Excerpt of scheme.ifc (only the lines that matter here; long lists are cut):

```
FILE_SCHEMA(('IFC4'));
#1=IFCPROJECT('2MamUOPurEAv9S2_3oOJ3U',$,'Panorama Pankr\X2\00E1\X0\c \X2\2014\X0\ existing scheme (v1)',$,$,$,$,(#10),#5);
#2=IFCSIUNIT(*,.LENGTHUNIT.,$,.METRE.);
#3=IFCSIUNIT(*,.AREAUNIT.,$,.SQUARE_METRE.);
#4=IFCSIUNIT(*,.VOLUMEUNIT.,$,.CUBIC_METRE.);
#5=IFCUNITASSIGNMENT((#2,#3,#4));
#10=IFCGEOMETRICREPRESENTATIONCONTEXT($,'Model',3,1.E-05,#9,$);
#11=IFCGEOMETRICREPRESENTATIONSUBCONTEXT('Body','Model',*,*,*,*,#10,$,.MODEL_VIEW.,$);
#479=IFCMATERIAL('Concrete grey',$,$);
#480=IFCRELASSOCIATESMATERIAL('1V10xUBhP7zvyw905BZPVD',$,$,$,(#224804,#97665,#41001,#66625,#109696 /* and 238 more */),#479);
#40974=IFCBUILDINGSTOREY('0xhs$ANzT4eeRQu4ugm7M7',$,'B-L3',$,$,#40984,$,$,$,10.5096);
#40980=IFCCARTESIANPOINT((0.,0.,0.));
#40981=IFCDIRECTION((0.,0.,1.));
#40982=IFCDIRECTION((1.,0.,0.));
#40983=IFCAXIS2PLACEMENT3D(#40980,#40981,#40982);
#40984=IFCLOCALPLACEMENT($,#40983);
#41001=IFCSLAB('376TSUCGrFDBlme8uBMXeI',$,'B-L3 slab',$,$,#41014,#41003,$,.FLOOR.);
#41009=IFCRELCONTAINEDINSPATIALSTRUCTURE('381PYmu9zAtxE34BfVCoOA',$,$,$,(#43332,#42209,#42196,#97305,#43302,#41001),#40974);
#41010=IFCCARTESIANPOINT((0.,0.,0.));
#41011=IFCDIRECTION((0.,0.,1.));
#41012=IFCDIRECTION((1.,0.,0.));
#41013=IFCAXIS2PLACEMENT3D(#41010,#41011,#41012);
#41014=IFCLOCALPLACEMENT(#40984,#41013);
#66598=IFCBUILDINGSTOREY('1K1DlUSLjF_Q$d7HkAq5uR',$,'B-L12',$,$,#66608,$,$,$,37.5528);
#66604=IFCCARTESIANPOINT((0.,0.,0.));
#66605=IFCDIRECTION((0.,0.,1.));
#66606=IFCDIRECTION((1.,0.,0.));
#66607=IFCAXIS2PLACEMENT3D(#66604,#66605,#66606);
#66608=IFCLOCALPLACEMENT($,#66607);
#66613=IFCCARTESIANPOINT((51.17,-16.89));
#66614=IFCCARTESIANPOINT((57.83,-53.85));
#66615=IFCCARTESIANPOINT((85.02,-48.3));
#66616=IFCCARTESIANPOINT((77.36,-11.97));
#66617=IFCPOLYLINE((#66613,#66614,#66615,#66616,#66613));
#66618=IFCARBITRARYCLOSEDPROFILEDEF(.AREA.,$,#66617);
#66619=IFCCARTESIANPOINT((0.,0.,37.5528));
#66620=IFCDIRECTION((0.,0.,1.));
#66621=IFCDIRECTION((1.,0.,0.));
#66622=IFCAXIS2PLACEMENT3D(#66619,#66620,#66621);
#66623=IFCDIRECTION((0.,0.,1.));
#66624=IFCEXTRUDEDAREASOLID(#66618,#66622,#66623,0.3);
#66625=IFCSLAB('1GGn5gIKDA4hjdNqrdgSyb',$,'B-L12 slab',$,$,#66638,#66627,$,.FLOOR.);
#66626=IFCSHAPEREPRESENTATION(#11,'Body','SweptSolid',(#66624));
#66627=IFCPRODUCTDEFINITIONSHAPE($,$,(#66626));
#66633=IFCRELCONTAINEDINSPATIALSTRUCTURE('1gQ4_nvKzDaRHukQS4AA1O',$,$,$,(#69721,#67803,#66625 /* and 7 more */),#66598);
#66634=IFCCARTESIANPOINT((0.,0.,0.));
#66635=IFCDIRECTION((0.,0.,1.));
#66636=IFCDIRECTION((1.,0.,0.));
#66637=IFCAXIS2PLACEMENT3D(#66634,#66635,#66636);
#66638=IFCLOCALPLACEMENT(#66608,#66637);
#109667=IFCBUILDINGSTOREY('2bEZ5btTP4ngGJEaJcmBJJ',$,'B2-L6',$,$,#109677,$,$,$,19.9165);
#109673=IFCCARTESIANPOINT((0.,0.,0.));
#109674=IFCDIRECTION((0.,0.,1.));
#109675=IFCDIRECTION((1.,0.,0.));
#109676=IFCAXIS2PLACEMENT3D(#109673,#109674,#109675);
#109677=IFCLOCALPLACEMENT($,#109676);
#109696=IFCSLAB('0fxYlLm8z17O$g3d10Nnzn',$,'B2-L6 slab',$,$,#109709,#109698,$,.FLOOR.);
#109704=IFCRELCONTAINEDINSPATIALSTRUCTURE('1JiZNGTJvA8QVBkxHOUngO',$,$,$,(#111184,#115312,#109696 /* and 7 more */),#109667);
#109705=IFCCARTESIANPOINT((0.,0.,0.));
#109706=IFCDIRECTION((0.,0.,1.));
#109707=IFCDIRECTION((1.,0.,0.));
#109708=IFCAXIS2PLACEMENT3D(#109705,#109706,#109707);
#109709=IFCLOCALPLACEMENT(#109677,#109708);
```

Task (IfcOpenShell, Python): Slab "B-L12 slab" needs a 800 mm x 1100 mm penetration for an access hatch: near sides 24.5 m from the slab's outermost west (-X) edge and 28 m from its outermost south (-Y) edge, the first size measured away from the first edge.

```python
import numpy as np
import ifcopenshell
import ifcopenshell.api.feature
import ifcopenshell.api.geometry
import ifcopenshell.api.root
import ifcopenshell.geom
import ifcopenshell.util.placement
import ifcopenshell.util.representation
import ifcopenshell.util.shape
import ifcopenshell.util.unit

model = ifcopenshell.open("scheme.ifc")
unit_scale = ifcopenshell.util.unit.calculate_unit_scale(model)
settings = ifcopenshell.geom.settings()


def volume(element):
    """Net volume in cubic metres, openings subtracted."""
    shape = ifcopenshell.geom.create_shape(settings, element)
    return ifcopenshell.util.shape.get_volume(shape.geometry)


slab = model.by_guid("1GGn5gIKDA4hjdNqrdgSyb")
before = volume(slab)

# Extent in the slab's own axes, in metres. The edges named are its -X and -Y sides.
slab_shape = ifcopenshell.geom.create_shape(settings, slab)
vertices = ifcopenshell.util.shape.get_vertices(slab_shape.geometry)
x_min, y_min, bottom = vertices.min(axis=0)
top = vertices[:, 2].max()

opening = ifcopenshell.api.root.create_entity(model, ifc_class="IfcOpeningElement", name="Access hatch opening", predefined_type="OPENING")
context = ifcopenshell.util.representation.get_context(model, "Model", "Body", "MODEL_VIEW")
width, depth = 0.8, 1.1
outline = [(0.0, 0.0), (width, 0.0), (width, depth), (0.0, depth), (0.0, 0.0)]
# Overshoot both faces by 50 mm so the cut is clean.
shape = ifcopenshell.api.geometry.add_slab_representation(
    model, context=context, depth=top - bottom + 0.1, polyline=outline
)
ifcopenshell.api.geometry.assign_representation(model, product=opening, representation=shape)

matrix = ifcopenshell.util.placement.get_local_placement(slab.ObjectPlacement)
matrix[:, 3] = matrix @ np.append(np.array([x_min + 24.5, y_min + 28, bottom - 0.05]) / unit_scale, 1.0)
ifcopenshell.api.geometry.edit_object_placement(model, product=opening, matrix=matrix, is_si=False)
ifcopenshell.api.feature.add_feature(model, feature=opening, element=slab)

after = volume(slab)

print(f"slab volume {before:.3f} -> {after:.3f} m3")

model.write("scheme_v2.ifc")
```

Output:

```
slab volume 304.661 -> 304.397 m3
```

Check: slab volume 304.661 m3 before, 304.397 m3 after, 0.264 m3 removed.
